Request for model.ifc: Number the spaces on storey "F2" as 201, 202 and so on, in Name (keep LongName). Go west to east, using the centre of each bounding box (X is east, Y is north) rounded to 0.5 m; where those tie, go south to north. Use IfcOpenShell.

First a look at what the model holds.

```python
import ifcopenshell
import ifcopenshell.util.element
import ifcopenshell.util.placement

model = ifcopenshell.open("model.ifc")
print(model.schema)
storey = next(s for s in model.by_type("IfcBuildingStorey") if s.Name == "F2")
spaces = [e for e in ifcopenshell.util.element.get_decomposition(storey) if e.is_a("IfcSpace")]
for e in sorted(spaces, key=lambda e: e.id()):
    origin = ifcopenshell.util.placement.get_local_placement(e.ObjectPlacement)[:3, 3]
    print(e.id(), e.Name, e.LongName, origin.round(2) + 0.0, sep=" | ")
```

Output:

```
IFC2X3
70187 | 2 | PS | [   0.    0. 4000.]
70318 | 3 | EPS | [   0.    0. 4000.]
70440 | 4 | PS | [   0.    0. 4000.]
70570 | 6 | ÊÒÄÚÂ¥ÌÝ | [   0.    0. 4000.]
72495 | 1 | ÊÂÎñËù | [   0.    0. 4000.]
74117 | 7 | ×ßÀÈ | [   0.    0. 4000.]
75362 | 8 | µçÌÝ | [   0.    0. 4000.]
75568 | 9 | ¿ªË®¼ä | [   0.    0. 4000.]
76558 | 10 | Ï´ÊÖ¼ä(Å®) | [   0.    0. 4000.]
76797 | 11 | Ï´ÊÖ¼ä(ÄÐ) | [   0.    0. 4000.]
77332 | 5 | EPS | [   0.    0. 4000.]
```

```python
import ifcopenshell
import ifcopenshell.geom
import ifcopenshell.util.element
import ifcopenshell.util.shape

model = ifcopenshell.open("model.ifc")
settings = ifcopenshell.geom.settings()
settings.set("use-world-coords", True)


def centre(element):
    shape = ifcopenshell.geom.create_shape(settings, element)
    return ifcopenshell.util.shape.get_bbox_centroid(shape.geometry)


storey = next(s for s in model.by_type("IfcBuildingStorey") if s.Name == "F2")
spaces = [e for e in ifcopenshell.util.element.get_decomposition(storey) if e.is_a("IfcSpace")]

# Insertion points can sit at a corner or the storey origin, so sort by the geometry (in metres).
centres = {e: centre(e) for e in spaces}
spaces.sort(key=lambda e: (round(centres[e][0] / 0.5), centres[e][1]))

for i, e in enumerate(spaces, start=1):
    number = f"2{i:02d}"
    e.Name = number
    print(e.id(), number)

model.write("model_edited.ifc")
```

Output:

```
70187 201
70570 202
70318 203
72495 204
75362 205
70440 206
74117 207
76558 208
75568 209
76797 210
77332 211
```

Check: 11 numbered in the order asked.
